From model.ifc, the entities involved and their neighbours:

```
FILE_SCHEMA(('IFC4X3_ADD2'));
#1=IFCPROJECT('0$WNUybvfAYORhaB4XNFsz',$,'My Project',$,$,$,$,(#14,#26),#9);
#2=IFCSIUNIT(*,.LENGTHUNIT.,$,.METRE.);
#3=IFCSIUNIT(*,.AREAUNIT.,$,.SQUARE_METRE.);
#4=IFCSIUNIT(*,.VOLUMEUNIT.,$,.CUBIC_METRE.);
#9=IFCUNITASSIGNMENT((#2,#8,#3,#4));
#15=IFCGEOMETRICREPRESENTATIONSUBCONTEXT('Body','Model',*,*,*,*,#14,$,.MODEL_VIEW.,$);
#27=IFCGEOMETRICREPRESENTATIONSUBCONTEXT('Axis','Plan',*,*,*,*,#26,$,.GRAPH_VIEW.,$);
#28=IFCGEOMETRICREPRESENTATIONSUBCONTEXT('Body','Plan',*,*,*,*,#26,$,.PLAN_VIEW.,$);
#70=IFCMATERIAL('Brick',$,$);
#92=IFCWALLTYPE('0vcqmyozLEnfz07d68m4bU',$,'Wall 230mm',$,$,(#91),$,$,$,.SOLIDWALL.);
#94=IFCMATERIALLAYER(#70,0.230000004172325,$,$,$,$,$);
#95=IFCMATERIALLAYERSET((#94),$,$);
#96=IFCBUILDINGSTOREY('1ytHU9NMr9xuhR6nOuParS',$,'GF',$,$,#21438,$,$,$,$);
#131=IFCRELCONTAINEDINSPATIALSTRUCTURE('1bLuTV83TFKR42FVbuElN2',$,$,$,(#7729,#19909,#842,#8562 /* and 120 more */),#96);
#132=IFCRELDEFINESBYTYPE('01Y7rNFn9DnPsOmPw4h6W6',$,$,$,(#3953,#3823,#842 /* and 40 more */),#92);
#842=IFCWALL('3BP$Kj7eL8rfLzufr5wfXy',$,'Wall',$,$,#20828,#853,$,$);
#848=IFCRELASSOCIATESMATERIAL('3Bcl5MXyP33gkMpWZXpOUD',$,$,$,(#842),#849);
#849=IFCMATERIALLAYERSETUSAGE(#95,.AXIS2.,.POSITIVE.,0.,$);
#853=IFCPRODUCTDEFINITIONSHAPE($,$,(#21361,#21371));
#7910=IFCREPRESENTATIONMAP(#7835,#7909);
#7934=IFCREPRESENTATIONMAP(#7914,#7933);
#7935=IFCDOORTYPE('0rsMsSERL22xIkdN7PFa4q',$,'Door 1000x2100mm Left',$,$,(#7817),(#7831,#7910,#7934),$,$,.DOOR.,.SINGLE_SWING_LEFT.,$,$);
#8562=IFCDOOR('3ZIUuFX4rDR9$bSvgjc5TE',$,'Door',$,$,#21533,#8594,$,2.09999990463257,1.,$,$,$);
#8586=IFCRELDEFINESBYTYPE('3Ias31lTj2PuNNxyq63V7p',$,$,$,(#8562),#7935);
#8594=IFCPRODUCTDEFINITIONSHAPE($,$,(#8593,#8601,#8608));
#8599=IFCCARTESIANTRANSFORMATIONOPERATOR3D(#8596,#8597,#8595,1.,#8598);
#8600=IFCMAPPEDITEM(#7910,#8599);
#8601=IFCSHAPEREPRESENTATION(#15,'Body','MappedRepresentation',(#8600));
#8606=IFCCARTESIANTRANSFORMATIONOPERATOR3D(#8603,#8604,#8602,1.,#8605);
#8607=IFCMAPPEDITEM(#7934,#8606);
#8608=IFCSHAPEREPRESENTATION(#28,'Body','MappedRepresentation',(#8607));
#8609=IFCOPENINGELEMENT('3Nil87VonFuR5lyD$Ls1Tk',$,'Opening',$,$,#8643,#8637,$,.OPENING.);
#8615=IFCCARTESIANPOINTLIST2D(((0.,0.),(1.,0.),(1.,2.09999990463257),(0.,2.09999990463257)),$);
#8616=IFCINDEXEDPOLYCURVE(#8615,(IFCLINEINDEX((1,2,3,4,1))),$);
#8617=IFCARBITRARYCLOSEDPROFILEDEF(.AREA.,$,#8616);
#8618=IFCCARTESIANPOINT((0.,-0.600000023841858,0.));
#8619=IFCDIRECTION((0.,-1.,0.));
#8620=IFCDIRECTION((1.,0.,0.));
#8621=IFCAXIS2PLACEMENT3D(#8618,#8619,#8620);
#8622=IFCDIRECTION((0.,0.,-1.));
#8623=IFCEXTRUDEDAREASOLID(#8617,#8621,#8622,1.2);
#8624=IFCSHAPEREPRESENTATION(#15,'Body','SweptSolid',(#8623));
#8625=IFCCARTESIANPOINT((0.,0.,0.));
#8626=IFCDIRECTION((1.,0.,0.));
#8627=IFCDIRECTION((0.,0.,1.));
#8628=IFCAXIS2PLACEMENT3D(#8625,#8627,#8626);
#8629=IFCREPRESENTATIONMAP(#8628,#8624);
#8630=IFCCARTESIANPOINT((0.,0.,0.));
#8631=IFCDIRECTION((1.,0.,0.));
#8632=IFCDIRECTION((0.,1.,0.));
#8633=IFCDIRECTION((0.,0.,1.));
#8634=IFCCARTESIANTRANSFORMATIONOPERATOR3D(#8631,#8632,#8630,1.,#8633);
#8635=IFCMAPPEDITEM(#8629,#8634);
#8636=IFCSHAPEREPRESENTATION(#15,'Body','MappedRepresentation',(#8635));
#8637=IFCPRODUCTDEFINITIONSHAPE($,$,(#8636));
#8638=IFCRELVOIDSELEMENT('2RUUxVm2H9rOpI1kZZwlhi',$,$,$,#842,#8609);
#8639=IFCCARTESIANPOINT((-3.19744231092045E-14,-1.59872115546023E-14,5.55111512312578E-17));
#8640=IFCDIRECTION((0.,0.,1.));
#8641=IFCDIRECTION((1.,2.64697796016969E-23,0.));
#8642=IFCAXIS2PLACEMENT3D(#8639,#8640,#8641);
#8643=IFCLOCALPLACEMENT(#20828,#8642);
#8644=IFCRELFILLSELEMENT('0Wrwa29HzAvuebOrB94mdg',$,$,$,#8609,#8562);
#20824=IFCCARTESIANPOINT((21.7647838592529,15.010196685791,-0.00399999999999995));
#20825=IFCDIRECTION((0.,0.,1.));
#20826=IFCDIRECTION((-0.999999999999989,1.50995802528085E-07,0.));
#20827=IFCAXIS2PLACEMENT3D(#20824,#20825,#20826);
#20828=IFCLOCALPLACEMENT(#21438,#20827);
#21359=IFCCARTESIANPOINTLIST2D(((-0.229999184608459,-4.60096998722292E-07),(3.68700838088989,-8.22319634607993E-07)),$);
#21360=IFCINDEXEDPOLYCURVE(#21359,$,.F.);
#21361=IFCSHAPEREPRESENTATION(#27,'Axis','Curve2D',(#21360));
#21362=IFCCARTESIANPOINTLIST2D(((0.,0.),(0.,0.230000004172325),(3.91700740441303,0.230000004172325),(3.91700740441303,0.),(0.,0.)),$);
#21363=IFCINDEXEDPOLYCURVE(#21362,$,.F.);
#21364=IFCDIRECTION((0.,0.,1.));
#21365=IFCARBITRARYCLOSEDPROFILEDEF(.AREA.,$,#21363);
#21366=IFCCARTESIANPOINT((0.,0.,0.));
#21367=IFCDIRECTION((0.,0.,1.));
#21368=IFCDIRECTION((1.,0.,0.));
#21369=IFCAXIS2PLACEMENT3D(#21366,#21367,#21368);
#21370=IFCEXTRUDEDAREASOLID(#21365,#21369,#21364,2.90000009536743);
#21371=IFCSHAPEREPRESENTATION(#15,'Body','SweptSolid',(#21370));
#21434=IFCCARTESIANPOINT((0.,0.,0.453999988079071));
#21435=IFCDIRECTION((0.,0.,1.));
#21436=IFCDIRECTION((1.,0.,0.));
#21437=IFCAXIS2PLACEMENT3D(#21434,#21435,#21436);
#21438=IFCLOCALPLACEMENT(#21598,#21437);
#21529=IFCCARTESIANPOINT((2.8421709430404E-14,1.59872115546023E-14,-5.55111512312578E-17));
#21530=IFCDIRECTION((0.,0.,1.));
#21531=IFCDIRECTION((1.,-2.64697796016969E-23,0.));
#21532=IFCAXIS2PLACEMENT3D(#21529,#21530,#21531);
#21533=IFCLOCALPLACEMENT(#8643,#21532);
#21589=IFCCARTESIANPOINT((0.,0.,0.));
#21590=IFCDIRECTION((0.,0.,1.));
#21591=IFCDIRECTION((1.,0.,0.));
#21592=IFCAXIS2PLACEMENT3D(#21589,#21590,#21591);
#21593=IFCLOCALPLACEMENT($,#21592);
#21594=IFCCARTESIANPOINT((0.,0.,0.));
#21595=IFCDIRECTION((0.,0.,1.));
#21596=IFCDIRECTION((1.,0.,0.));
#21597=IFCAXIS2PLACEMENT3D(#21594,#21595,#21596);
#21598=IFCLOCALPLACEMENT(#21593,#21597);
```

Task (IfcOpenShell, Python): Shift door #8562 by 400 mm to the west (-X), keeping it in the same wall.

```python
import ifcopenshell
import ifcopenshell.api.geometry
import ifcopenshell.util.placement
import ifcopenshell.util.unit

model = ifcopenshell.open("model.ifc")
unit_scale = ifcopenshell.util.unit.calculate_unit_scale(model)

door = model.by_guid("3ZIUuFX4rDR9$bSvgjc5TE")
opening = door.FillsVoids[0].RelatingOpeningElement
wall = opening.VoidsElements[0].RelatingBuildingElement

wall_matrix = ifcopenshell.util.placement.get_local_placement(wall.ObjectPlacement)
shift = wall_matrix[:3, 0] * 0.4 / unit_scale
before = ifcopenshell.util.placement.get_local_placement(door.ObjectPlacement)[:3, 3].copy()

# The door is placed relative to its opening, so it follows when the opening moves.
matrix = ifcopenshell.util.placement.get_local_placement(opening.ObjectPlacement)
matrix[:3, 3] += shift
ifcopenshell.api.geometry.edit_object_placement(
    model, product=opening, matrix=matrix, is_si=False, should_transform_children=True
)

after = ifcopenshell.util.placement.get_local_placement(door.ObjectPlacement)[:3, 3]
print("door moved by", (after - before).round(3) + 0.0)

model.write("model_edited.ifc")
```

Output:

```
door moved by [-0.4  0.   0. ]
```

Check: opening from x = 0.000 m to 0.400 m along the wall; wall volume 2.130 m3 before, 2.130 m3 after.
